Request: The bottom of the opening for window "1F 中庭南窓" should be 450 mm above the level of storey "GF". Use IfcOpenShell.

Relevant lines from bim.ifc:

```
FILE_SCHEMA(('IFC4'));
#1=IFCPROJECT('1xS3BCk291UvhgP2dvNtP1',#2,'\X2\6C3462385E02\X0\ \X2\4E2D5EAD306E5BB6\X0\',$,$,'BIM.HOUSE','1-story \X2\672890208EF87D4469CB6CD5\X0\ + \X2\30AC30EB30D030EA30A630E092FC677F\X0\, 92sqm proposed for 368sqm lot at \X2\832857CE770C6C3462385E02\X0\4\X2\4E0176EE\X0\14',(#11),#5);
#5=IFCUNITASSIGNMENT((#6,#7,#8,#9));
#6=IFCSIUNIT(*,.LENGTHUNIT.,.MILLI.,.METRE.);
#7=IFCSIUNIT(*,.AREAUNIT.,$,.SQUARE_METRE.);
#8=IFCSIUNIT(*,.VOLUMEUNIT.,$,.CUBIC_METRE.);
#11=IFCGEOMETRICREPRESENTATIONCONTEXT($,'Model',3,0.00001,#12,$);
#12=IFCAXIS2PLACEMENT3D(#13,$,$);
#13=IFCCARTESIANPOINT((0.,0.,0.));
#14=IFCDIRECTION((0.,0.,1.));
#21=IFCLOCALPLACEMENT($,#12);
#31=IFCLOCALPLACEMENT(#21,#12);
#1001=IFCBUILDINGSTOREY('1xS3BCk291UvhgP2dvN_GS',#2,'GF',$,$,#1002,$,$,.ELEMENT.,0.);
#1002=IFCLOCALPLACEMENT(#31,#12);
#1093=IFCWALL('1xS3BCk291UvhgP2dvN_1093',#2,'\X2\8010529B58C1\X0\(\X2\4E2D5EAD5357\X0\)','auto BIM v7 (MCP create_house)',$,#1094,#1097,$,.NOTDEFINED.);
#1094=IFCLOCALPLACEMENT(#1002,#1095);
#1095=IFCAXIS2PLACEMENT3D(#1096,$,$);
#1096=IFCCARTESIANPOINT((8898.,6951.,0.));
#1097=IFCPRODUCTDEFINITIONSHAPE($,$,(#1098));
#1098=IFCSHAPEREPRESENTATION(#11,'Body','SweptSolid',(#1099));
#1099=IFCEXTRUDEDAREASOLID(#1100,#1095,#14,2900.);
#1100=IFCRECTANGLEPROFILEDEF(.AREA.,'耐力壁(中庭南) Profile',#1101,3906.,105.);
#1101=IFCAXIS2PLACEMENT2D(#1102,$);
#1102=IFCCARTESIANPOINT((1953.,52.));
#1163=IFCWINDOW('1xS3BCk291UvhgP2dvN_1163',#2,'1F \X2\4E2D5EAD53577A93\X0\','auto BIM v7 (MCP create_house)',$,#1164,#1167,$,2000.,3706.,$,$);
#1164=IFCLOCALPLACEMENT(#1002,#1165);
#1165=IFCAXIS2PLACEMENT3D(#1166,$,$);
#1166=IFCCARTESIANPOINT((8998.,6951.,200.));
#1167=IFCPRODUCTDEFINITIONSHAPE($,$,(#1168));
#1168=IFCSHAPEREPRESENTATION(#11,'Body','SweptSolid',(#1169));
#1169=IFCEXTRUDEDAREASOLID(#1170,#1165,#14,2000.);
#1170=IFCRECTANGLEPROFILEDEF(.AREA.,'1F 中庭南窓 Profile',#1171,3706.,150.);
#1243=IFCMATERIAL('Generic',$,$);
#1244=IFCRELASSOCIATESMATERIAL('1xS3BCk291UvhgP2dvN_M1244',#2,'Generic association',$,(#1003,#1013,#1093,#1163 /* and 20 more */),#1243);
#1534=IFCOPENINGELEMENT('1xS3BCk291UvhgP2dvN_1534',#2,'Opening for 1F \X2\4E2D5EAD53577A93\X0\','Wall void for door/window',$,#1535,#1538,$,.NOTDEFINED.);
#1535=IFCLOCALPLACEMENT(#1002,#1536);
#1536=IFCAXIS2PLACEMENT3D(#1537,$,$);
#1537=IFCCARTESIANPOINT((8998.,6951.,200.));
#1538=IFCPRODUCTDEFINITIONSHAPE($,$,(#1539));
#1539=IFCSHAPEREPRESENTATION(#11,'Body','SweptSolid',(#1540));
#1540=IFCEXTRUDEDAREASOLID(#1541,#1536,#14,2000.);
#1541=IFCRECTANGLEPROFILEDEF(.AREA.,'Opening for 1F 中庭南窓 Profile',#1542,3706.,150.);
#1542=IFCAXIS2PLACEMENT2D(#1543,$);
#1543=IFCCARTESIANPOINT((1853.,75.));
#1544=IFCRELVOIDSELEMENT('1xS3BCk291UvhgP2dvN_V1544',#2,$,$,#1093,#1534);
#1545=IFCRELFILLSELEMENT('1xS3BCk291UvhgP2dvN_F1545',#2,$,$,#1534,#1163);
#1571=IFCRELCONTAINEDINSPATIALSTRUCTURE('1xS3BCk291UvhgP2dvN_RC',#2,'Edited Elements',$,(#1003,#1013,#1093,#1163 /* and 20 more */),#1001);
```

```python
import numpy as np
import ifcopenshell
import ifcopenshell.api.geometry
import ifcopenshell.geom
import ifcopenshell.util.element
import ifcopenshell.util.placement
import ifcopenshell.util.shape
import ifcopenshell.util.unit

model = ifcopenshell.open("bim.ifc")
unit_scale = ifcopenshell.util.unit.calculate_unit_scale(model)

window = model.by_guid("1xS3BCk291UvhgP2dvN_1163")
opening = window.FillsVoids[0].RelatingOpeningElement
storey = ifcopenshell.util.element.get_container(window, ifc_class="IfcBuildingStorey")
level = ifcopenshell.util.placement.get_local_placement(storey.ObjectPlacement)[2, 3]

# The opening's origin need not be at the sill, so measure its lowest point.
shape = ifcopenshell.geom.create_shape(ifcopenshell.geom.settings(), opening)
bottom = ifcopenshell.util.shape.get_shape_bottom_elevation(shape, shape.geometry) / unit_scale
dz = level + 0.45 / unit_scale - bottom

shift = np.array([0.0, 0.0, dz])
# The window is not placed relative to its opening, so move both.
for product in (opening, window):
    matrix = ifcopenshell.util.placement.get_local_placement(product.ObjectPlacement)
    matrix[:3, 3] += shift
    ifcopenshell.api.geometry.edit_object_placement(model, product=product, matrix=matrix, is_si=False)

print(f"moved by {dz * unit_scale:+.3f} m")

model.write("bim_v2.ifc")
```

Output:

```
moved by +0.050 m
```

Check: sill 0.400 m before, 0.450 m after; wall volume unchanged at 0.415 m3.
